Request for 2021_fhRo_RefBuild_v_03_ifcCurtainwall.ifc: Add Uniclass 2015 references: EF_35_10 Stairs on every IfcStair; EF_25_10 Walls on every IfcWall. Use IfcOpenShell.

First a look at what the model holds.

```python
import ifcopenshell

model = ifcopenshell.open("2021_fhRo_RefBuild_v_03_ifcCurtainwall.ifc")
print(model.schema)
print("classifications:", [c.Name for c in model.by_type("IfcClassification")])
for ifc_class in ("IfcDoor", "IfcRoof", "IfcStair", "IfcWall", "IfcWindow"):
    print(ifc_class, len(model.by_type(ifc_class)))
```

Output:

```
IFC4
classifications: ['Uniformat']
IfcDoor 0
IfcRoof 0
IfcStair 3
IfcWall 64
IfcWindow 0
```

```python
import ifcopenshell
import ifcopenshell.api.classification

model = ifcopenshell.open("2021_fhRo_RefBuild_v_03_ifcCurtainwall.ifc")

system = ifcopenshell.api.classification.add_classification(model, classification="Uniclass 2015")

codes = {
    "IfcStair": ("EF_35_10", "Stairs"),
    "IfcWall": ("EF_25_10", "Walls"),
}
for ifc_class, (code, name) in codes.items():
    products = model.by_type(ifc_class)
    ifcopenshell.api.classification.add_reference(
        model, products=products, classification=system, identification=code, name=name
    )
    print(code, len(products))

model.write("2021_fhRo_RefBuild_v_03_ifcCurtainwall-out.ifc")
```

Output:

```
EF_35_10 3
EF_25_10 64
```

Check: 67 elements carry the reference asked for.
